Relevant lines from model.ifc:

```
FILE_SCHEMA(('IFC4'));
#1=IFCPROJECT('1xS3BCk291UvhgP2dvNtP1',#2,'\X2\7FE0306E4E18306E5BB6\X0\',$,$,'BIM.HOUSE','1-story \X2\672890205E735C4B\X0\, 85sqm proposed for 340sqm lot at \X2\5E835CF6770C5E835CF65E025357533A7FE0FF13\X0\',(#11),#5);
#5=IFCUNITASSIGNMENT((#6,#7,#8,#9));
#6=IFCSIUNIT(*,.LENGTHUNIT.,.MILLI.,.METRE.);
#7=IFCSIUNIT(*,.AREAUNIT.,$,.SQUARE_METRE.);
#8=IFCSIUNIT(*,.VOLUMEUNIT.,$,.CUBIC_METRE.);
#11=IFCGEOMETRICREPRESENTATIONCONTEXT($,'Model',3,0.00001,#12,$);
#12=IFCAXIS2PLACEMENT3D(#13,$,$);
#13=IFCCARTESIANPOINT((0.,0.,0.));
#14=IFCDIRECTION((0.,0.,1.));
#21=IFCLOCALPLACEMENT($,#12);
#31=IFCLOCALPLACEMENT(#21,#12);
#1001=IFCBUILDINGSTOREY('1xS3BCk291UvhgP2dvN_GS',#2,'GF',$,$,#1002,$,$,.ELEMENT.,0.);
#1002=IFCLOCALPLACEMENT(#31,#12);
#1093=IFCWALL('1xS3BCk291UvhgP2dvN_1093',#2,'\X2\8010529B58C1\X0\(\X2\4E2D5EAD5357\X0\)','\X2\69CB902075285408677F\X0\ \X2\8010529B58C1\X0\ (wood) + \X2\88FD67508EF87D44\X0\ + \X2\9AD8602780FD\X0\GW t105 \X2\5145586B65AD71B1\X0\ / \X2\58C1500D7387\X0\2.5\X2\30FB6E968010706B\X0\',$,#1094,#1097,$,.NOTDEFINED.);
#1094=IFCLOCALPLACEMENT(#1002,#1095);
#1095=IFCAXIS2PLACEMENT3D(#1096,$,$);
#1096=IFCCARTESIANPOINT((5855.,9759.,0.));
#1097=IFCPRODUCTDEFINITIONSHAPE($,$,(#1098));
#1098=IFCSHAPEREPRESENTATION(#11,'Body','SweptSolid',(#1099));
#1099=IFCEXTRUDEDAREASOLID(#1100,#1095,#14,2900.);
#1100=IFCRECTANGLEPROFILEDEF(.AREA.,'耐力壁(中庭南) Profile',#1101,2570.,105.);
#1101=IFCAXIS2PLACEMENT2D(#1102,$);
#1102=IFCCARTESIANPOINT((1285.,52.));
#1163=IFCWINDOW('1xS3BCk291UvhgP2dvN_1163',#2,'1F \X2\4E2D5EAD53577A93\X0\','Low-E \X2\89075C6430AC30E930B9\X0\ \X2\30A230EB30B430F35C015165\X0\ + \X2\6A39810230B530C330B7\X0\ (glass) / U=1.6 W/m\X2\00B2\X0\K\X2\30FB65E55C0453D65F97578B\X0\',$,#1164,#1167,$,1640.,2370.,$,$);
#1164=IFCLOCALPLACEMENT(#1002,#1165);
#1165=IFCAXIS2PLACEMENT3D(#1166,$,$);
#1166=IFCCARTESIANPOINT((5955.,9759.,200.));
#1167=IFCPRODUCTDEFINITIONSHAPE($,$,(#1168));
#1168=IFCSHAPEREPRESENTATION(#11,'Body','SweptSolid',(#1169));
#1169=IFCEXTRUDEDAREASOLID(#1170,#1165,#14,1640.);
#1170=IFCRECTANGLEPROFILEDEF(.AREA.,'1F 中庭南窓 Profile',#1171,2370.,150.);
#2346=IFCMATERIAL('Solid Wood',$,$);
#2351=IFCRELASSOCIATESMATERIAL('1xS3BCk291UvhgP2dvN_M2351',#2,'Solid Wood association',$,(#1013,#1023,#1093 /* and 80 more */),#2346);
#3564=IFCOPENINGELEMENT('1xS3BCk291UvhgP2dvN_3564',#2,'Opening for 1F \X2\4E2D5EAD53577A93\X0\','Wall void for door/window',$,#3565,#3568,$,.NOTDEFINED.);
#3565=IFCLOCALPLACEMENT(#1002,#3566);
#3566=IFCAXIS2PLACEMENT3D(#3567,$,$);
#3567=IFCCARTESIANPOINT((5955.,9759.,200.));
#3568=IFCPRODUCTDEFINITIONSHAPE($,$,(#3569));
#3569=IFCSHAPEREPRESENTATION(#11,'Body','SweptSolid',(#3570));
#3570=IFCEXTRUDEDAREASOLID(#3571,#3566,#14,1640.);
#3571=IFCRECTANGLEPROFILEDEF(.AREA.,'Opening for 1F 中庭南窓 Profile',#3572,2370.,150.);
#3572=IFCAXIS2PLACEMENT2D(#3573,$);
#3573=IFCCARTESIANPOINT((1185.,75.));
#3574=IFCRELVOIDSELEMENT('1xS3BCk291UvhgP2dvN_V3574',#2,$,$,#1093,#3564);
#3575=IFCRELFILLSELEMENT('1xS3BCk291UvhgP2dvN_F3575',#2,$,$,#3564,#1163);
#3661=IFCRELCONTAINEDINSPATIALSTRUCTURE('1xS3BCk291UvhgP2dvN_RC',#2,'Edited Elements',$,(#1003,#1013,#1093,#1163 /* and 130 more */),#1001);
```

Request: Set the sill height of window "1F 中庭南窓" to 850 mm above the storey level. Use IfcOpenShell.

```python
import numpy as np
import ifcopenshell
import ifcopenshell.api.geometry
import ifcopenshell.geom
import ifcopenshell.util.element
import ifcopenshell.util.placement
import ifcopenshell.util.shape
import ifcopenshell.util.unit

model = ifcopenshell.open("model.ifc")
unit_scale = ifcopenshell.util.unit.calculate_unit_scale(model)

window = model.by_guid("1xS3BCk291UvhgP2dvN_1163")
opening = window.FillsVoids[0].RelatingOpeningElement
storey = ifcopenshell.util.element.get_container(window, ifc_class="IfcBuildingStorey")
level = ifcopenshell.util.placement.get_local_placement(storey.ObjectPlacement)[2, 3]

# The opening's origin need not be at the sill, so measure its lowest point.
shape = ifcopenshell.geom.create_shape(ifcopenshell.geom.settings(), opening)
bottom = ifcopenshell.util.shape.get_shape_bottom_elevation(shape, shape.geometry) / unit_scale
dz = level + 0.85 / unit_scale - bottom

shift = np.array([0.0, 0.0, dz])
# The window is not placed relative to its opening, so move both.
for product in (opening, window):
    matrix = ifcopenshell.util.placement.get_local_placement(product.ObjectPlacement)
    matrix[:3, 3] += shift
    ifcopenshell.api.geometry.edit_object_placement(model, product=product, matrix=matrix, is_si=False)

print(f"moved by {dz * unit_scale:+.3f} m")

model.write("model_updated.ifc")
```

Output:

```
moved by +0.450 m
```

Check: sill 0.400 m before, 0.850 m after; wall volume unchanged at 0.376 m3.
